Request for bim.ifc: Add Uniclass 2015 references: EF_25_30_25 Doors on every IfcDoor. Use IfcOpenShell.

First a look at what the model holds.

```python
import ifcopenshell

model = ifcopenshell.open("bim.ifc")
print(model.schema)
print("classifications:", [c.Name for c in model.by_type("IfcClassification")])
for ifc_class in ("IfcDoor", "IfcRoof", "IfcStair", "IfcWall", "IfcWindow"):
    print(ifc_class, len(model.by_type(ifc_class)))
```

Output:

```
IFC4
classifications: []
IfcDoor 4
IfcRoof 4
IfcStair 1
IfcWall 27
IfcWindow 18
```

```python
import ifcopenshell
import ifcopenshell.api.classification

model = ifcopenshell.open("bim.ifc")

system = ifcopenshell.api.classification.add_classification(model, classification="Uniclass 2015")

codes = {
    "IfcDoor": ("EF_25_30_25", "Doors"),
}
for ifc_class, (code, name) in codes.items():
    products = model.by_type(ifc_class)
    ifcopenshell.api.classification.add_reference(
        model, products=products, classification=system, identification=code, name=name
    )
    print(code, len(products))

model.write("bim_edited.ifc")
```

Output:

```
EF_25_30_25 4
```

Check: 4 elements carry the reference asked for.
